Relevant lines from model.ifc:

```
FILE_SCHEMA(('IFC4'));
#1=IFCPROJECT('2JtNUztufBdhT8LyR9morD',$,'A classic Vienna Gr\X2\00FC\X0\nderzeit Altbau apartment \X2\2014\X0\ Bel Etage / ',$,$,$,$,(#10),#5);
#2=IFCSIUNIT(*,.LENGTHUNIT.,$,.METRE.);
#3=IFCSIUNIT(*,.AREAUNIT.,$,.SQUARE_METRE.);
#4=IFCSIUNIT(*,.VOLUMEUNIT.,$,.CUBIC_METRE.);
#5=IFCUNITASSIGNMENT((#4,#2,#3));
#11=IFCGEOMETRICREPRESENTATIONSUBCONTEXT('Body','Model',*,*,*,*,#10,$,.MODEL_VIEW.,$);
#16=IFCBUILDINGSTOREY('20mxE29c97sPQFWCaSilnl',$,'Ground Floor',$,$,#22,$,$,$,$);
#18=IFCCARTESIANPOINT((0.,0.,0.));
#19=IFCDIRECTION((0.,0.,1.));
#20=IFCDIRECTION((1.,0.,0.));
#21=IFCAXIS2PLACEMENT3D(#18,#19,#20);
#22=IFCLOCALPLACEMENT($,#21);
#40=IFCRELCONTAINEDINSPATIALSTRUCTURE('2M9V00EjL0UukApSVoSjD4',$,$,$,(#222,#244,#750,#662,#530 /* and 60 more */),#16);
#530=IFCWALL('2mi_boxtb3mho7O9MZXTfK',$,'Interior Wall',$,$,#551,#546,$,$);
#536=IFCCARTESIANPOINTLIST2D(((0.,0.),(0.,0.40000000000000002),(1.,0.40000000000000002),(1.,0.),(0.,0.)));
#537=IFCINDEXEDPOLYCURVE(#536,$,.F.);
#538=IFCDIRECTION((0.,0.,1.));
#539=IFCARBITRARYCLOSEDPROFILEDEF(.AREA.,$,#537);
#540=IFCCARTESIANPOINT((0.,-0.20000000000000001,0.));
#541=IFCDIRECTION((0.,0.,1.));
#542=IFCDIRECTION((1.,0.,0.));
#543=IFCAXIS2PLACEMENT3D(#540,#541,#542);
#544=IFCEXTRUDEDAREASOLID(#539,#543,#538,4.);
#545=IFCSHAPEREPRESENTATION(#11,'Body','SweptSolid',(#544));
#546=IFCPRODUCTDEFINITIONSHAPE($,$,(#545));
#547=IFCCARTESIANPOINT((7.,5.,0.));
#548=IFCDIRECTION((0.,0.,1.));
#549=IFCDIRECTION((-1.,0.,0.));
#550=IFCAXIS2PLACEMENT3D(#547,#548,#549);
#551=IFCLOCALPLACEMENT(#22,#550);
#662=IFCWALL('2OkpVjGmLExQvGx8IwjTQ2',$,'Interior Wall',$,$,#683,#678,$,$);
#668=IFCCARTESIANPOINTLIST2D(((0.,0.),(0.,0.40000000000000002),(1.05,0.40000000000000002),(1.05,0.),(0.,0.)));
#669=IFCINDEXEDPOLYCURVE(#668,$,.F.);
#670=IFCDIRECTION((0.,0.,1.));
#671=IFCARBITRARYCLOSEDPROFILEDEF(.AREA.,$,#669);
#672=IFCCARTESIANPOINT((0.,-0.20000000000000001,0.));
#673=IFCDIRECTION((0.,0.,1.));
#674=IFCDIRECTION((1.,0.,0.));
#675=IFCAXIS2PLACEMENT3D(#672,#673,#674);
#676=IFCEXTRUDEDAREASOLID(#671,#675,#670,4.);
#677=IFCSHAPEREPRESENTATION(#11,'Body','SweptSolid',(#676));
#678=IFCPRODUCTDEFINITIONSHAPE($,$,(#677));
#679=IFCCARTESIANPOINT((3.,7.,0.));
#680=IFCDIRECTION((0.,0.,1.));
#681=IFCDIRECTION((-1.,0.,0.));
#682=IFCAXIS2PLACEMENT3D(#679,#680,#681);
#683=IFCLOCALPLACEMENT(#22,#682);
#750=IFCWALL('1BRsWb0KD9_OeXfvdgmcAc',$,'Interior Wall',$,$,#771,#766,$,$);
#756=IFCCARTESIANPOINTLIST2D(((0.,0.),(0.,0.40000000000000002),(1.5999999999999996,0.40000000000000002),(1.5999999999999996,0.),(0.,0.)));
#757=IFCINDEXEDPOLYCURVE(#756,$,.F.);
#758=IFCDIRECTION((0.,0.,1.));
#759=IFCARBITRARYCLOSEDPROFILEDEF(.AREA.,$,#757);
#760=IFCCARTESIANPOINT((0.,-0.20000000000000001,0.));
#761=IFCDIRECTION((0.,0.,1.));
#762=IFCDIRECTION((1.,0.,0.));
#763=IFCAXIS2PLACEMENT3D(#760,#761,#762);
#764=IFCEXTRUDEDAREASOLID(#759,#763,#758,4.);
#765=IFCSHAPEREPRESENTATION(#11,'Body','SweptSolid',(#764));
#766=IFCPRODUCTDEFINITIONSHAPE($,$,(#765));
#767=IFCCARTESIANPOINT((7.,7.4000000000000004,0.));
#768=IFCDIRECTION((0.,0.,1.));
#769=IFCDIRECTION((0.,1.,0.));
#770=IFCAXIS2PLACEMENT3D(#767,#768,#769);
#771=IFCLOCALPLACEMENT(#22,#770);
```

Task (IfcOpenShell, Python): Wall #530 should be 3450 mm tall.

```python
import ifcopenshell
import ifcopenshell.geom
import ifcopenshell.util.representation
import ifcopenshell.util.shape
import ifcopenshell.util.unit

model = ifcopenshell.open("model.ifc")
unit_scale = ifcopenshell.util.unit.calculate_unit_scale(model)
settings = ifcopenshell.geom.settings()


def volume(element):
    """Net volume in cubic metres, openings subtracted."""
    shape = ifcopenshell.geom.create_shape(settings, element)
    return ifcopenshell.util.shape.get_volume(shape.geometry)


wall = model.by_id(530)
before = volume(wall)

body = ifcopenshell.util.representation.get_representation(wall, "Model", "Body")
solid = body.Items[0]
old_height = solid.Depth
solid.Depth = 3.45 / unit_scale
after = volume(wall)

print(f"height {old_height:g} -> {solid.Depth:g}, volume {before:.3f} -> {after:.3f} m3")

model.write("model-out.ifc")
```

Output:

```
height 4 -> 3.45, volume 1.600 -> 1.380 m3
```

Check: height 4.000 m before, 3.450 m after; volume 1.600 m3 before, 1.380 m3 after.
